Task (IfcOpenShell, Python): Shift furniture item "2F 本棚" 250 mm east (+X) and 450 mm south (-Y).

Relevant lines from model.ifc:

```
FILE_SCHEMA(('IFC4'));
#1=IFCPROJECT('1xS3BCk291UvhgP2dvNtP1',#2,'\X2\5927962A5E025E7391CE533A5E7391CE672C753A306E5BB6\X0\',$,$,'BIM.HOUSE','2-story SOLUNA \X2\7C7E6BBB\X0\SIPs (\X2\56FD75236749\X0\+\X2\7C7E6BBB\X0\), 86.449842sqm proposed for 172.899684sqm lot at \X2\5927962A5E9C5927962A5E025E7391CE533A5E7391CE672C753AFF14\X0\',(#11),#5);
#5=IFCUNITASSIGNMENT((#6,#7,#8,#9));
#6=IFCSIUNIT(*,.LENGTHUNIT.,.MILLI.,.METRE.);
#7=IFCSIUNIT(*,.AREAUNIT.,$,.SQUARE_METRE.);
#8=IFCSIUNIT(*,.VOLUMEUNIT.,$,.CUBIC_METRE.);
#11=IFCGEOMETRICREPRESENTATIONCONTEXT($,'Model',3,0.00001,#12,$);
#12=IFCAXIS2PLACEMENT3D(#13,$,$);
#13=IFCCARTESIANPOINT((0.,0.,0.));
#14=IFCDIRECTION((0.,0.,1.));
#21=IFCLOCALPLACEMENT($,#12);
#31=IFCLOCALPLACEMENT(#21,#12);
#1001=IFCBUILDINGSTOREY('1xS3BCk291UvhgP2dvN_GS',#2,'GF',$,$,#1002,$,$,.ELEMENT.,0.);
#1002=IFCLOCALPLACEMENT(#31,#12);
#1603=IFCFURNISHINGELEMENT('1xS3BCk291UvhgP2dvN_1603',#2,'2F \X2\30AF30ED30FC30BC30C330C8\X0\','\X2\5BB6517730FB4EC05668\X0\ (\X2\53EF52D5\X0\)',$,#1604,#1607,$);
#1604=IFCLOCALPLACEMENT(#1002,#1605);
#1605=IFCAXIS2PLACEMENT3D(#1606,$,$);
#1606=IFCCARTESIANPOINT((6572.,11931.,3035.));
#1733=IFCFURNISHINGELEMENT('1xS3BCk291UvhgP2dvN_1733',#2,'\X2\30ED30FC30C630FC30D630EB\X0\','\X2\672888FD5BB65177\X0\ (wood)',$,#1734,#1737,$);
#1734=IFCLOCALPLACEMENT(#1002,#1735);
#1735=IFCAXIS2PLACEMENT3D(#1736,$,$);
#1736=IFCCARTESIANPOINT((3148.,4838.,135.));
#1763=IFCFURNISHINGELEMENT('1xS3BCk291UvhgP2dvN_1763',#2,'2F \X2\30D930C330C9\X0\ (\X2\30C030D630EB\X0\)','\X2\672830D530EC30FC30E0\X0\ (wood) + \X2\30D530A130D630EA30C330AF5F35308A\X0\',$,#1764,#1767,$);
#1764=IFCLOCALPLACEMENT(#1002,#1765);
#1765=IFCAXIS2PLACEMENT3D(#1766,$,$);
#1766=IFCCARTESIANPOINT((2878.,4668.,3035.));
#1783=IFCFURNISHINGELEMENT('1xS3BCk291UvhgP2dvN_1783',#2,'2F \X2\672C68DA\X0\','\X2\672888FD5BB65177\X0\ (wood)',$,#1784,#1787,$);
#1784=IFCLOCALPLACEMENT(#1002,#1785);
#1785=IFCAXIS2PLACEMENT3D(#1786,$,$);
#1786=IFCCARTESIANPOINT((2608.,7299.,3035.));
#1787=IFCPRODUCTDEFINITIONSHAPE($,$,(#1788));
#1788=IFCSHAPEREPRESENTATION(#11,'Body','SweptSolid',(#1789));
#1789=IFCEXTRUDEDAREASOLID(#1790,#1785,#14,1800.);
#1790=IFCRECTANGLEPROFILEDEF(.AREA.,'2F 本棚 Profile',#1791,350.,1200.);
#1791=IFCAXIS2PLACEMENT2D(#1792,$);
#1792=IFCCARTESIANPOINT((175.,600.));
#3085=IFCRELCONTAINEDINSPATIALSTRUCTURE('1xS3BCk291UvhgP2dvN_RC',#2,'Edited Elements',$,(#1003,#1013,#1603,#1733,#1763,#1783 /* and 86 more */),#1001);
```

```python
import ifcopenshell
import ifcopenshell.api.geometry
import ifcopenshell.util.placement
import ifcopenshell.util.unit

model = ifcopenshell.open("model.ifc")
unit_scale = ifcopenshell.util.unit.calculate_unit_scale(model)

item = model.by_guid("1xS3BCk291UvhgP2dvN_1783")
matrix = ifcopenshell.util.placement.get_local_placement(item.ObjectPlacement)
matrix[0, 3] += 0.25 / unit_scale
matrix[1, 3] -= 0.45 / unit_scale
ifcopenshell.api.geometry.edit_object_placement(model, product=item, matrix=matrix, is_si=False)

print(ifcopenshell.util.placement.get_local_placement(item.ObjectPlacement).round(3) + 0.0)

model.write("model-out.ifc")
```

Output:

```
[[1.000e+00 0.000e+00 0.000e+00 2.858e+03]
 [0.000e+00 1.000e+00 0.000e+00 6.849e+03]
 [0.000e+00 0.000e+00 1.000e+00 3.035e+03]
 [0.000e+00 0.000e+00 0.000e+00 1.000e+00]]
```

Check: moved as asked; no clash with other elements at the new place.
